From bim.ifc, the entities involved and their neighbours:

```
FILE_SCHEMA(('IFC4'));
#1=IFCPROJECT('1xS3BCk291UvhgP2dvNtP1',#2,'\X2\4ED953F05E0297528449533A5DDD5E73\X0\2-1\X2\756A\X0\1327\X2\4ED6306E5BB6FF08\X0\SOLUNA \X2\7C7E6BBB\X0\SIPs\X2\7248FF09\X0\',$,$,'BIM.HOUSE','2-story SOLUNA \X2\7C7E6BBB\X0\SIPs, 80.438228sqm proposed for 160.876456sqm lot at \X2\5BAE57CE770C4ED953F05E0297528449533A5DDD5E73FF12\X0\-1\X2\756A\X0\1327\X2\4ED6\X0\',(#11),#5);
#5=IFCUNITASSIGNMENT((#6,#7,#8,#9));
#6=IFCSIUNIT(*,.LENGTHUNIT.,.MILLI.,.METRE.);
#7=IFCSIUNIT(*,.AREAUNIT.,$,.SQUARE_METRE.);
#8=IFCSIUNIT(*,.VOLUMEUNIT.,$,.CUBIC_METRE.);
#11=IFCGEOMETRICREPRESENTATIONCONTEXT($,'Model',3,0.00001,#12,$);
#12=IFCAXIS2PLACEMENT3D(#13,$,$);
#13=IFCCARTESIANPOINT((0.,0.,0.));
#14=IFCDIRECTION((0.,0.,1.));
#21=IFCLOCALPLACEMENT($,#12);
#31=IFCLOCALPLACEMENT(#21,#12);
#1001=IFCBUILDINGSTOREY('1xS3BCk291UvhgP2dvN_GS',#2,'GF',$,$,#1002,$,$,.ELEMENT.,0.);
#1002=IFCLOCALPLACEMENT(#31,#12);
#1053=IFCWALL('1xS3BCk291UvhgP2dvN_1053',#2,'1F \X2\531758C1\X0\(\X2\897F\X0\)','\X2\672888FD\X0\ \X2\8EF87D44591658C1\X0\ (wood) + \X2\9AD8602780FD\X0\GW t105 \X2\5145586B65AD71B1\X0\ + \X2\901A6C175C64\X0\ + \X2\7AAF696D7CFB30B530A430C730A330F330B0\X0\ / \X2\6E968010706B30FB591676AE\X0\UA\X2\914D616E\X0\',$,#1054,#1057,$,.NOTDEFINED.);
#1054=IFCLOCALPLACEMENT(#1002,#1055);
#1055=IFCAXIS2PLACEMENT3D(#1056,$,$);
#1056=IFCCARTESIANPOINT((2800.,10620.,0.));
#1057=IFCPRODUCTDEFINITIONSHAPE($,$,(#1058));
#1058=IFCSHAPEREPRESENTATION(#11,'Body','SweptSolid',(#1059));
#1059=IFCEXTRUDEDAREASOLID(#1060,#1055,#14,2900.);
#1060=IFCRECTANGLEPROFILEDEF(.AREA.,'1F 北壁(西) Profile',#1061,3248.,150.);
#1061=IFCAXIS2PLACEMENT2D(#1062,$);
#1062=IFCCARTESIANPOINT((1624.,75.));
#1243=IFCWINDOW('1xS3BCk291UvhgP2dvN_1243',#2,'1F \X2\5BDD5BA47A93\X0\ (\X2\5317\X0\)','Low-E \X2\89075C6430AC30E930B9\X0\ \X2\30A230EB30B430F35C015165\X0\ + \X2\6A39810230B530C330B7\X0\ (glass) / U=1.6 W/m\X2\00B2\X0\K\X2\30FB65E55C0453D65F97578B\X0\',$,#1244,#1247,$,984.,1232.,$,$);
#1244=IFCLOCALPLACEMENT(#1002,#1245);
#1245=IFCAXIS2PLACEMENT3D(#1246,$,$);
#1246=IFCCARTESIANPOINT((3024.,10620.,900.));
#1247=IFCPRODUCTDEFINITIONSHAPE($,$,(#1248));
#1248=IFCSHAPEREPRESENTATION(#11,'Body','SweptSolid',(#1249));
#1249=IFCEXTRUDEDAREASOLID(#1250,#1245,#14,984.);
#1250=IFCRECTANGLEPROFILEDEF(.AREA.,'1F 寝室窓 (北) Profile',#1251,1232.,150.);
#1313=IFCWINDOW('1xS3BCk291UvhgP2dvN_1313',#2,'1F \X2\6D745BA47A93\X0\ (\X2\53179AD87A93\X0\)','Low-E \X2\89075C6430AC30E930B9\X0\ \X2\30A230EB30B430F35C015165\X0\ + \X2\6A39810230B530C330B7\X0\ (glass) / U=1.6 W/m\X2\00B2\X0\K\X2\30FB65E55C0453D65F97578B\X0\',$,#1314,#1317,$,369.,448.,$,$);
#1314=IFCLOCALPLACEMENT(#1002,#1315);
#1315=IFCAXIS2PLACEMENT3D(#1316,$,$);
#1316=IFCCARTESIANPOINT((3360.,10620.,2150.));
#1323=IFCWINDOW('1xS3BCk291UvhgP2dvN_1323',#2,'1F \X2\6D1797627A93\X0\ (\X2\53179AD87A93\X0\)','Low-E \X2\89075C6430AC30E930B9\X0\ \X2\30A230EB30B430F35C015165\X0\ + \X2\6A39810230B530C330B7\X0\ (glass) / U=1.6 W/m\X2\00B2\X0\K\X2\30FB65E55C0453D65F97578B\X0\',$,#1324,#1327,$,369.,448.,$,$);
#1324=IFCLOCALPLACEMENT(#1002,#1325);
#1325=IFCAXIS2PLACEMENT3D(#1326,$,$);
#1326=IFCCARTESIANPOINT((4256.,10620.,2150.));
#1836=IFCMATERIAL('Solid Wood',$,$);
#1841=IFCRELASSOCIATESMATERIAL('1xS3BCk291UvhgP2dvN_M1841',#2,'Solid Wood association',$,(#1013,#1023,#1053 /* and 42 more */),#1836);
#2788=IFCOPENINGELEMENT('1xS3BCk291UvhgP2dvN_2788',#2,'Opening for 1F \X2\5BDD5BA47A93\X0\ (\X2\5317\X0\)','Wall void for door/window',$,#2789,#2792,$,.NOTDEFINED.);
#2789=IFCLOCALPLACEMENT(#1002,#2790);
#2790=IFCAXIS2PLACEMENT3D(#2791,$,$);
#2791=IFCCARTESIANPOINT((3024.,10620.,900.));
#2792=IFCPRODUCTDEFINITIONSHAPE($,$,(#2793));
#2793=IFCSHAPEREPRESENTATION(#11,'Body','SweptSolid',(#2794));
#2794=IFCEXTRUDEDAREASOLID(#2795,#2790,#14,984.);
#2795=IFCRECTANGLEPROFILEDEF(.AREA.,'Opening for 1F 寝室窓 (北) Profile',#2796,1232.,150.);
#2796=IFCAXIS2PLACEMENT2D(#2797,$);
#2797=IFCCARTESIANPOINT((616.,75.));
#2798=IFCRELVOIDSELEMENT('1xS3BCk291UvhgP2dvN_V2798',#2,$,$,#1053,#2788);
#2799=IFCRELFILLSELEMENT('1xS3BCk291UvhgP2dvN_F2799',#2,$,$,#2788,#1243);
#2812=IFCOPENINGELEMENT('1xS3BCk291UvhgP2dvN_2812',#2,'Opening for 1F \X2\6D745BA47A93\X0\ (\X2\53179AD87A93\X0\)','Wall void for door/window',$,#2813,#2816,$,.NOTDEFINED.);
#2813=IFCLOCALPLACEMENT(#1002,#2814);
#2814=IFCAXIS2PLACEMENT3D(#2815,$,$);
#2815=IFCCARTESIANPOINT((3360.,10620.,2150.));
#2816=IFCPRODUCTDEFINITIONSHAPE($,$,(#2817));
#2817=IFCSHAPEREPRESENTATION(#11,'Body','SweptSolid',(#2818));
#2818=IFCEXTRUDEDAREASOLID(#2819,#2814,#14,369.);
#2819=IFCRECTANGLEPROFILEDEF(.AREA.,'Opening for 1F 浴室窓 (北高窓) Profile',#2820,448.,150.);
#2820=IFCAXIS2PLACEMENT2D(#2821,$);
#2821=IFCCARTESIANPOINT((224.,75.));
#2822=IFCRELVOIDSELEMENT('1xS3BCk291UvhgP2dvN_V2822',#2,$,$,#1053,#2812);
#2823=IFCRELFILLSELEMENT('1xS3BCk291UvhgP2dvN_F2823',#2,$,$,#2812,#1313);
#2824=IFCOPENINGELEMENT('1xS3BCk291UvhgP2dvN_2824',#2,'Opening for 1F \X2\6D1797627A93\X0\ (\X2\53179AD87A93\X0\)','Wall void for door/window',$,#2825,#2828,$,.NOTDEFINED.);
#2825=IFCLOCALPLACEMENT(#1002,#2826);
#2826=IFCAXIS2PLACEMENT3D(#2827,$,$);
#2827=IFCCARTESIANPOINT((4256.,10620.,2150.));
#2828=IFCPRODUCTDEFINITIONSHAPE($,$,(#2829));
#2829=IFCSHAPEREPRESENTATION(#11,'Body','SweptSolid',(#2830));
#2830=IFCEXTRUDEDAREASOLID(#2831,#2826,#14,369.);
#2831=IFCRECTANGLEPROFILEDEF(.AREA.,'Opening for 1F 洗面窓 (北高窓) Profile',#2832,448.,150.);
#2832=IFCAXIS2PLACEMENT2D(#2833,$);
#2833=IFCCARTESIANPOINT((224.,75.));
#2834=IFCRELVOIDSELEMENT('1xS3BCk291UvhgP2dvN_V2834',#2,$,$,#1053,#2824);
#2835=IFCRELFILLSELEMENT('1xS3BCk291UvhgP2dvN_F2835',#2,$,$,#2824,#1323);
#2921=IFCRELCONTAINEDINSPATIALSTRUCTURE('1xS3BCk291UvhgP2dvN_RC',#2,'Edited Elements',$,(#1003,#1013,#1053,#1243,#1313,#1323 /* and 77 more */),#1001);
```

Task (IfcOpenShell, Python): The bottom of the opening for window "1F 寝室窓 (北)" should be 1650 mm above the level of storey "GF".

```python
import numpy as np
import ifcopenshell
import ifcopenshell.api.geometry
import ifcopenshell.geom
import ifcopenshell.util.element
import ifcopenshell.util.placement
import ifcopenshell.util.shape
import ifcopenshell.util.unit

model = ifcopenshell.open("bim.ifc")
unit_scale = ifcopenshell.util.unit.calculate_unit_scale(model)

window = model.by_guid("1xS3BCk291UvhgP2dvN_1243")
opening = window.FillsVoids[0].RelatingOpeningElement
storey = ifcopenshell.util.element.get_container(window, ifc_class="IfcBuildingStorey")
level = ifcopenshell.util.placement.get_local_placement(storey.ObjectPlacement)[2, 3]

# The opening's origin need not be at the sill, so measure its lowest point.
shape = ifcopenshell.geom.create_shape(ifcopenshell.geom.settings(), opening)
bottom = ifcopenshell.util.shape.get_shape_bottom_elevation(shape, shape.geometry) / unit_scale
dz = level + 1.65 / unit_scale - bottom

shift = np.array([0.0, 0.0, dz])
# The window is not placed relative to its opening, so move both.
for product in (opening, window):
    matrix = ifcopenshell.util.placement.get_local_placement(product.ObjectPlacement)
    matrix[:3, 3] += shift
    ifcopenshell.api.geometry.edit_object_placement(model, product=product, matrix=matrix, is_si=False)

print(f"moved by {dz * unit_scale:+.3f} m")

model.write("bim_updated.ifc")
```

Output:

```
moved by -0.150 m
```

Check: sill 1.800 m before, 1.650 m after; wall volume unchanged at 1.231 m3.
